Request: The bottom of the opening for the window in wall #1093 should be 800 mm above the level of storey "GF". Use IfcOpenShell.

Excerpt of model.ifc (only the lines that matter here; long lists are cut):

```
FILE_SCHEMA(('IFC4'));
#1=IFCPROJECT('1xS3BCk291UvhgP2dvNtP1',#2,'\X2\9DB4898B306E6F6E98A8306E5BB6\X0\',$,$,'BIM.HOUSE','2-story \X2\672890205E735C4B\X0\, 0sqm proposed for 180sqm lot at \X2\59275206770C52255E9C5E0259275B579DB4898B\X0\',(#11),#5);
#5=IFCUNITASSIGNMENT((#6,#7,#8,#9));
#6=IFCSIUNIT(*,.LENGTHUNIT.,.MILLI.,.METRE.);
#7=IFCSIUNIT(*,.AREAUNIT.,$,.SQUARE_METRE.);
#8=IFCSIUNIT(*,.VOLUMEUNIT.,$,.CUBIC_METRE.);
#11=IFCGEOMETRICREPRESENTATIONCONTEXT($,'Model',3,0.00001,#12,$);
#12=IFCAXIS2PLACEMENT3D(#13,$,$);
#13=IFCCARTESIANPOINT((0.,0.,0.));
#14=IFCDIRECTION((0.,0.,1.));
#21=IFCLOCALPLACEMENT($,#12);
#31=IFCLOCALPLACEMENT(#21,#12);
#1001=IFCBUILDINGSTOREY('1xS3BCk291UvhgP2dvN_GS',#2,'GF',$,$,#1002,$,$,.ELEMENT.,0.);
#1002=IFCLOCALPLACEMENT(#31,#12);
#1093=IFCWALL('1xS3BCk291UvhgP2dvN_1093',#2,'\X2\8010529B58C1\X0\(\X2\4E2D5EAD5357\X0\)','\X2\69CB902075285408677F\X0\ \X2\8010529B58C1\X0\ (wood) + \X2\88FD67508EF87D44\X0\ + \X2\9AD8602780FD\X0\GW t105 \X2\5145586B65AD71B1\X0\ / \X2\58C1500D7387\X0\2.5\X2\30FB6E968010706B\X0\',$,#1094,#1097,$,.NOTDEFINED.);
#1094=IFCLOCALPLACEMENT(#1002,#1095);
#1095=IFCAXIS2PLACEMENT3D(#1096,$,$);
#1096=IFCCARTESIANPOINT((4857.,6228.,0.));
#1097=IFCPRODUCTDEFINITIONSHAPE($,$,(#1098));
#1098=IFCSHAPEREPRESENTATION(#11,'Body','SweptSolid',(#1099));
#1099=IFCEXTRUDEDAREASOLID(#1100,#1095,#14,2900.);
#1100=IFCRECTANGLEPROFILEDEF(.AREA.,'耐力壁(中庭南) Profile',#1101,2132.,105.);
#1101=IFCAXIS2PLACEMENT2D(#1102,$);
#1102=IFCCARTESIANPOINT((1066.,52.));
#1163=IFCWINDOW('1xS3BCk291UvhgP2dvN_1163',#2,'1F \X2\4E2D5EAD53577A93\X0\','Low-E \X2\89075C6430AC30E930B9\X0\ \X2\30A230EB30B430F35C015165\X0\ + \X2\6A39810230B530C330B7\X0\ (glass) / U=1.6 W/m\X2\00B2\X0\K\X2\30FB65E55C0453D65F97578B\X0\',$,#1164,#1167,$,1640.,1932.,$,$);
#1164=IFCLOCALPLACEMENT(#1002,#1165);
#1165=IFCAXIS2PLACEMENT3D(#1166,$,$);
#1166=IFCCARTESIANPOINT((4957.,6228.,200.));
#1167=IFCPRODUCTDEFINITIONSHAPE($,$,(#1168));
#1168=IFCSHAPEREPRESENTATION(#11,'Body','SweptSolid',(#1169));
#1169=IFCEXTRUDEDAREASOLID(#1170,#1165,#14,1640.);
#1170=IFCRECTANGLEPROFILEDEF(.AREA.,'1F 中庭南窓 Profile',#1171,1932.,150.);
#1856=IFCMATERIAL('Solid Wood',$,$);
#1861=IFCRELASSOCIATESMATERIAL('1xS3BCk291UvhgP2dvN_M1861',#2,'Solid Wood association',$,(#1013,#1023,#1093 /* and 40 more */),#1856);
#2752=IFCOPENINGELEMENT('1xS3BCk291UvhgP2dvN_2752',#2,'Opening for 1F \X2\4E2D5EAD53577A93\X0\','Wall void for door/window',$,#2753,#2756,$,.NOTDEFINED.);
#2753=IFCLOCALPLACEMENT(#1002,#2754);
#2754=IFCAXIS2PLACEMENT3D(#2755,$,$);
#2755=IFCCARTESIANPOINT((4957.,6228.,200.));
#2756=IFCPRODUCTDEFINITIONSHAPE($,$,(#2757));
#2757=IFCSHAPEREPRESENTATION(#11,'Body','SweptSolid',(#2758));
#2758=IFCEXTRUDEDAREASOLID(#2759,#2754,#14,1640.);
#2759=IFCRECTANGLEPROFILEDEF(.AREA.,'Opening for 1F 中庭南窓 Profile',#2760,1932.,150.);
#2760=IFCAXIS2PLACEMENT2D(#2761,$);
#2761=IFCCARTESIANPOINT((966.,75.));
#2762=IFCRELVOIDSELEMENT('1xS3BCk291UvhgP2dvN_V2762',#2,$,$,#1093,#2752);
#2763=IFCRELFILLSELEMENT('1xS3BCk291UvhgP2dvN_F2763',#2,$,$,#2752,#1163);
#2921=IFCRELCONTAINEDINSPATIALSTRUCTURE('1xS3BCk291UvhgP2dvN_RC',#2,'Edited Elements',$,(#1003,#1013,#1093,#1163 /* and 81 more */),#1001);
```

```python
import numpy as np
import ifcopenshell
import ifcopenshell.api.geometry
import ifcopenshell.geom
import ifcopenshell.util.element
import ifcopenshell.util.placement
import ifcopenshell.util.shape
import ifcopenshell.util.unit

model = ifcopenshell.open("model.ifc")
unit_scale = ifcopenshell.util.unit.calculate_unit_scale(model)

window = model.by_guid("1xS3BCk291UvhgP2dvN_1163")
opening = window.FillsVoids[0].RelatingOpeningElement
storey = ifcopenshell.util.element.get_container(window, ifc_class="IfcBuildingStorey")
level = ifcopenshell.util.placement.get_local_placement(storey.ObjectPlacement)[2, 3]

# The opening's origin need not be at the sill, so measure its lowest point.
shape = ifcopenshell.geom.create_shape(ifcopenshell.geom.settings(), opening)
bottom = ifcopenshell.util.shape.get_shape_bottom_elevation(shape, shape.geometry) / unit_scale
dz = level + 0.8 / unit_scale - bottom

shift = np.array([0.0, 0.0, dz])
# The window is not placed relative to its opening, so move both.
for product in (opening, window):
    matrix = ifcopenshell.util.placement.get_local_placement(product.ObjectPlacement)
    matrix[:3, 3] += shift
    ifcopenshell.api.geometry.edit_object_placement(model, product=product, matrix=matrix, is_si=False)

print(f"moved by {dz * unit_scale:+.3f} m")

model.write("model_edited.ifc")
```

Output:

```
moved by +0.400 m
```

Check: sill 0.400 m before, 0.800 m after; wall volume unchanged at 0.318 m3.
